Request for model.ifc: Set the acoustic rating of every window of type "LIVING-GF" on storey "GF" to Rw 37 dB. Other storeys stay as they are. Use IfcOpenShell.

First a look at what the model holds.

```python
import ifcopenshell
import ifcopenshell.util.element

model = ifcopenshell.open("model.ifc")
print(model.schema)
storey = next(s for s in model.by_type("IfcBuildingStorey") if s.Name == "GF")
windows = [e for e in ifcopenshell.util.element.get_decomposition(storey) if e.is_a("IfcWindow")]
seen = {}
for e in windows:
    element_type = ifcopenshell.util.element.get_type(e)
    key = (element_type.Name if element_type != e and element_type else None, ifcopenshell.util.element.get_pset(e, "Pset_WindowCommon", "AcousticRating"))
    seen[key] = seen.get(key, 0) + 1
for (name, value), count in sorted(seen.items(), key=str):
    print(count, "x", name, "|", value)
```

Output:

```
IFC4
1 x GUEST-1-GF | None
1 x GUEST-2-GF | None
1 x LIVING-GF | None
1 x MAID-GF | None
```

```python
import ifcopenshell
import ifcopenshell.api.pset
import ifcopenshell.util.element

model = ifcopenshell.open("model.ifc")

storey = next(s for s in model.by_type("IfcBuildingStorey") if s.Name == "GF")
windows = [e for e in ifcopenshell.util.element.get_decomposition(storey) if e.is_a("IfcWindow")]

count = 0
for e in windows:
    element_type = ifcopenshell.util.element.get_type(e)
    if element_type in (None, e) or element_type.Name != "LIVING-GF":
        continue
    # add_pset returns the element's existing set when there is one.
    pset = ifcopenshell.api.pset.add_pset(model, product=e, name="Pset_WindowCommon")
    ifcopenshell.api.pset.edit_pset(model, pset=pset, properties={"AcousticRating": "Rw 37 dB"})
    count += 1

print(count, "windows updated")

model.write("model_v2.ifc")
```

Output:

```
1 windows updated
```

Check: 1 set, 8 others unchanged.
